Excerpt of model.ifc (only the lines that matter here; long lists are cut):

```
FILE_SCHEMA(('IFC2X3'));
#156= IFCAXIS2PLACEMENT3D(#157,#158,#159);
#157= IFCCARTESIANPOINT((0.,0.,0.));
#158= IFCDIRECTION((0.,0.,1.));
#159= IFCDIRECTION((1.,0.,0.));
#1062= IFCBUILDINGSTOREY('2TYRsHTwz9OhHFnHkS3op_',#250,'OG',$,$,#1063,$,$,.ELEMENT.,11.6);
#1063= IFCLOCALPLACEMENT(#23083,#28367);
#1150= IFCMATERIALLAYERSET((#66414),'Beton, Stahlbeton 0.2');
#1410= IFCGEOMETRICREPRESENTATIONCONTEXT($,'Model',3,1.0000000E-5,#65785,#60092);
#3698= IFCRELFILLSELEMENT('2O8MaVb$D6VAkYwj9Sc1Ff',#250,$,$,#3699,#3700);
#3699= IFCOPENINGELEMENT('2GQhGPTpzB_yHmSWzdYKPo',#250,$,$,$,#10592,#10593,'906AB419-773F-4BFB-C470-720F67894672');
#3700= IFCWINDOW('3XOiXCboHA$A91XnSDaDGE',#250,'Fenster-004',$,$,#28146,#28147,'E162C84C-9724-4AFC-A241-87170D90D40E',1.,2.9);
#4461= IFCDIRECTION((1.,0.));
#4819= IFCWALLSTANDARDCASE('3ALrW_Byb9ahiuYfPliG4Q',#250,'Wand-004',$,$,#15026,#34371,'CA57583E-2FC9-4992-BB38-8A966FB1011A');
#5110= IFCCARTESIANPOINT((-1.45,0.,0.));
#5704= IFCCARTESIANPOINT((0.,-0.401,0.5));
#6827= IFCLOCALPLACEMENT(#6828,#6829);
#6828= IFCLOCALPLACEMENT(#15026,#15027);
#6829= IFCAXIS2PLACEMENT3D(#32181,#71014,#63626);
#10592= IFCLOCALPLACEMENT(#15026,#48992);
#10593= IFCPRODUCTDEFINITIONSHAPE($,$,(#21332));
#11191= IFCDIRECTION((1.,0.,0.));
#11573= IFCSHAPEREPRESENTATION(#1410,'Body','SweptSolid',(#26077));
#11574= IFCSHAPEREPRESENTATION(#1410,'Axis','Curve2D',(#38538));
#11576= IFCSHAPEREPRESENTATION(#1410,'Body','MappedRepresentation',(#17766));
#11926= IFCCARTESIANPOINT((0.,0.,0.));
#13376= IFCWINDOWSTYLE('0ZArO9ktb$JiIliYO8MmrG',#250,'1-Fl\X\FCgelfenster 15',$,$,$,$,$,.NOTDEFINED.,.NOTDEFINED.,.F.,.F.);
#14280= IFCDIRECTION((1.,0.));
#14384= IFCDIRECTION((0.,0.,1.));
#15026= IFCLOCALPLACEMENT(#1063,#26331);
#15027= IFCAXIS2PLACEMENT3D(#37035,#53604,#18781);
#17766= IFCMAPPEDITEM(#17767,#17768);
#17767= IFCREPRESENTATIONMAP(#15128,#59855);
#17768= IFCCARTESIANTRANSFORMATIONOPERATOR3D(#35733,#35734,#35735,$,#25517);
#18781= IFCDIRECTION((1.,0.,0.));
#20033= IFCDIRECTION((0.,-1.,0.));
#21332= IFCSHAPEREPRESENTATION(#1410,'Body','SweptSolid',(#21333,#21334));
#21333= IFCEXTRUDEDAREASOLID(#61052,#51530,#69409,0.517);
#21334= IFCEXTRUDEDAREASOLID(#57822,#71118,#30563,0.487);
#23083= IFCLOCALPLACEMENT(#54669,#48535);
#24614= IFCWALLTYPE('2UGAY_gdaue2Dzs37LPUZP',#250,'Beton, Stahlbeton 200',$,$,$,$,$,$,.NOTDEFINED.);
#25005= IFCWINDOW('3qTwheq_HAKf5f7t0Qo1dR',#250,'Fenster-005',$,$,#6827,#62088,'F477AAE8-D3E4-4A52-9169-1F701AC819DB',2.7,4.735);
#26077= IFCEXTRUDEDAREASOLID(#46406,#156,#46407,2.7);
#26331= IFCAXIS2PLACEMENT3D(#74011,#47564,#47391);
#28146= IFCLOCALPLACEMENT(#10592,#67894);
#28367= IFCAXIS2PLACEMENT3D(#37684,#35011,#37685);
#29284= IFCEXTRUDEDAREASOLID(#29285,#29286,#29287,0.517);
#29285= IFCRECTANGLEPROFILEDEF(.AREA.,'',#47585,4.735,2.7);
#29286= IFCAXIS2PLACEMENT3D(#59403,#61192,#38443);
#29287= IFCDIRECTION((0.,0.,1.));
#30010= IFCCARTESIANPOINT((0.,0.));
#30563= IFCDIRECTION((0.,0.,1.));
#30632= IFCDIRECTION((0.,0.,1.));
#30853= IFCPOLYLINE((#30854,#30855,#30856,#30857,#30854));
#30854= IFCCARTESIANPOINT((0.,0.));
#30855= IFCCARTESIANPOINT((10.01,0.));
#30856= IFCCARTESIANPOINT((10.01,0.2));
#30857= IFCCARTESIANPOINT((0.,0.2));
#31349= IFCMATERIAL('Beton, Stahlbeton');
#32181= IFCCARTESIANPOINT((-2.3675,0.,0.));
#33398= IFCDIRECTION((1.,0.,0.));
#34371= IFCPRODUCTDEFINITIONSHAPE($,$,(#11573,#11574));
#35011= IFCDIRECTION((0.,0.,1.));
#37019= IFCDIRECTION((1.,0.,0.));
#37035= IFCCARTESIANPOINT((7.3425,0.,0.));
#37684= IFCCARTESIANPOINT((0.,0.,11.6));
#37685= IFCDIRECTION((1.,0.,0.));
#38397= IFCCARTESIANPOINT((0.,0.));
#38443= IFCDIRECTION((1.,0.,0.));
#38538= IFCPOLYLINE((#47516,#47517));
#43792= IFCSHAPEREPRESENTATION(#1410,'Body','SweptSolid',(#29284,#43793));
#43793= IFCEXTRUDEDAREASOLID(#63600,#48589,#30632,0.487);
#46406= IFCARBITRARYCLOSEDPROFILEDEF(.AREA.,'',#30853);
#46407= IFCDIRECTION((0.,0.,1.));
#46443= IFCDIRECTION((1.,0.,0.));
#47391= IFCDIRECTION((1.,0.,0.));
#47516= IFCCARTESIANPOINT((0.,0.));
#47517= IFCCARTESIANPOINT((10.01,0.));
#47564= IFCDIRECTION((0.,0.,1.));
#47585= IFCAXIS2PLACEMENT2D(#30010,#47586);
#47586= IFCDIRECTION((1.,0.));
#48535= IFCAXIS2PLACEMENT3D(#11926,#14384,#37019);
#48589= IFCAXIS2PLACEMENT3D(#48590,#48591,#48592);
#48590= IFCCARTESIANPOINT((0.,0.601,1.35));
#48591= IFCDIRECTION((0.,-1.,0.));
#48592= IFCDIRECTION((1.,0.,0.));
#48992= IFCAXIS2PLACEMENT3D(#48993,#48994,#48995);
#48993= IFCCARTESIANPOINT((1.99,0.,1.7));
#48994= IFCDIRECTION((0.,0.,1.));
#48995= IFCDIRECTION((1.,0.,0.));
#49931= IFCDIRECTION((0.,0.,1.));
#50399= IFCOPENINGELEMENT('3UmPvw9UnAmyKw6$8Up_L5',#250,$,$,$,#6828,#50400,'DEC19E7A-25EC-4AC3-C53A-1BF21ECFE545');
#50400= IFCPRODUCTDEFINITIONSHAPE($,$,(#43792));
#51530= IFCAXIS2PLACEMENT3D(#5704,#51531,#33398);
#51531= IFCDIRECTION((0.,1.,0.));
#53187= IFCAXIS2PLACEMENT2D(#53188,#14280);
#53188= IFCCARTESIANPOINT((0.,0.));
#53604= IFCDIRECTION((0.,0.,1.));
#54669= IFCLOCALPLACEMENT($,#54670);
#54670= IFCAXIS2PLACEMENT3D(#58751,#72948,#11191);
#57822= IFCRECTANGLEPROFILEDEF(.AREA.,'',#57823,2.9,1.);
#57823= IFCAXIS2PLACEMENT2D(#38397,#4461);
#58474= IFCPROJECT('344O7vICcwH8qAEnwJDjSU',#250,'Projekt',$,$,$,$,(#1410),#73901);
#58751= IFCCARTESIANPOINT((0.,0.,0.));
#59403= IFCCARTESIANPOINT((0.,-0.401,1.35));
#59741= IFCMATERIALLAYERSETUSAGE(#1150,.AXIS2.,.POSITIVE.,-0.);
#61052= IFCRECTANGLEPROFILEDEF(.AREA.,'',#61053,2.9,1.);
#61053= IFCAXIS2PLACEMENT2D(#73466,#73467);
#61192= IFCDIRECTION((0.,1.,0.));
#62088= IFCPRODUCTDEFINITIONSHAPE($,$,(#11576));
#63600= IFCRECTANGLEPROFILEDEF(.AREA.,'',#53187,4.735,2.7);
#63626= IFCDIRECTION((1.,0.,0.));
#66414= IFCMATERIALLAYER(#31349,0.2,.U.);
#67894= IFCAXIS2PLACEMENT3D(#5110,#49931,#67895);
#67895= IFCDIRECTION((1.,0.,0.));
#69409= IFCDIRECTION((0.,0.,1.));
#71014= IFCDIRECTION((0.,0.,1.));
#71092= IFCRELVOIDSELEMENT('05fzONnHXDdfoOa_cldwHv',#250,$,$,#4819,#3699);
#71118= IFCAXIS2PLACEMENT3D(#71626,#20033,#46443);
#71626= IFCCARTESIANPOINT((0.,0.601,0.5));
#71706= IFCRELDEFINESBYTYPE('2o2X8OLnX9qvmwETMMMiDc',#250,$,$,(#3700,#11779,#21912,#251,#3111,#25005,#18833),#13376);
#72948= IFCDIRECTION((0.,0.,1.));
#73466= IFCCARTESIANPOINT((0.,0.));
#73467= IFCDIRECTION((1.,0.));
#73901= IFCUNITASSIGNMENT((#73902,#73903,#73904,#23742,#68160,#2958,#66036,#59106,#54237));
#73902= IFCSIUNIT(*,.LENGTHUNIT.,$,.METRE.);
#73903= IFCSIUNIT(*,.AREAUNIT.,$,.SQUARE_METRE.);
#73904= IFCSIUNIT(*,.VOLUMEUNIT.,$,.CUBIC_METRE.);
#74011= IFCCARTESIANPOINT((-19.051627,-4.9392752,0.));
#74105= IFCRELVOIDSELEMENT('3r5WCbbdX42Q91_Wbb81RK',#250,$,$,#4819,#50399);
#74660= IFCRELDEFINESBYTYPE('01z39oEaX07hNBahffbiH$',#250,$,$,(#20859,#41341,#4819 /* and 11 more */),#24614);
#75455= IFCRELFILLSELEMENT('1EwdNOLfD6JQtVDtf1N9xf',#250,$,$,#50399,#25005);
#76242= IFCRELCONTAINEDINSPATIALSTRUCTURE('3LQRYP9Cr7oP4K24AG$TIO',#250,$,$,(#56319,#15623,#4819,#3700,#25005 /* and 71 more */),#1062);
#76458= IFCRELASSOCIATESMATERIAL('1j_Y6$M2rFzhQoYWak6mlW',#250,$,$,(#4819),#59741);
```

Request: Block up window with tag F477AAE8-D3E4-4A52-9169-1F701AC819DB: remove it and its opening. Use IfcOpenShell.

```python
import ifcopenshell
import ifcopenshell.api.feature
import ifcopenshell.api.root
import ifcopenshell.geom
import ifcopenshell.util.shape

model = ifcopenshell.open("model.ifc")
settings = ifcopenshell.geom.settings()


def volume(element):
    """Net volume in cubic metres, openings subtracted."""
    shape = ifcopenshell.geom.create_shape(settings, element)
    return ifcopenshell.util.shape.get_volume(shape.geometry)


window = model.by_id(25005)
opening = window.FillsVoids[0].RelatingOpeningElement
wall = opening.VoidsElements[0].RelatingBuildingElement
before = volume(wall)

ifcopenshell.api.root.remove_product(model, product=window)
ifcopenshell.api.feature.remove_feature(model, feature=opening)

after = volume(wall)

print(f"wall volume {before:.3f} -> {after:.3f} m3")

model.write("model_edited.ifc")
```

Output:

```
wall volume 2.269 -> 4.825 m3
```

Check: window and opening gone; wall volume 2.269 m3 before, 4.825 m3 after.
